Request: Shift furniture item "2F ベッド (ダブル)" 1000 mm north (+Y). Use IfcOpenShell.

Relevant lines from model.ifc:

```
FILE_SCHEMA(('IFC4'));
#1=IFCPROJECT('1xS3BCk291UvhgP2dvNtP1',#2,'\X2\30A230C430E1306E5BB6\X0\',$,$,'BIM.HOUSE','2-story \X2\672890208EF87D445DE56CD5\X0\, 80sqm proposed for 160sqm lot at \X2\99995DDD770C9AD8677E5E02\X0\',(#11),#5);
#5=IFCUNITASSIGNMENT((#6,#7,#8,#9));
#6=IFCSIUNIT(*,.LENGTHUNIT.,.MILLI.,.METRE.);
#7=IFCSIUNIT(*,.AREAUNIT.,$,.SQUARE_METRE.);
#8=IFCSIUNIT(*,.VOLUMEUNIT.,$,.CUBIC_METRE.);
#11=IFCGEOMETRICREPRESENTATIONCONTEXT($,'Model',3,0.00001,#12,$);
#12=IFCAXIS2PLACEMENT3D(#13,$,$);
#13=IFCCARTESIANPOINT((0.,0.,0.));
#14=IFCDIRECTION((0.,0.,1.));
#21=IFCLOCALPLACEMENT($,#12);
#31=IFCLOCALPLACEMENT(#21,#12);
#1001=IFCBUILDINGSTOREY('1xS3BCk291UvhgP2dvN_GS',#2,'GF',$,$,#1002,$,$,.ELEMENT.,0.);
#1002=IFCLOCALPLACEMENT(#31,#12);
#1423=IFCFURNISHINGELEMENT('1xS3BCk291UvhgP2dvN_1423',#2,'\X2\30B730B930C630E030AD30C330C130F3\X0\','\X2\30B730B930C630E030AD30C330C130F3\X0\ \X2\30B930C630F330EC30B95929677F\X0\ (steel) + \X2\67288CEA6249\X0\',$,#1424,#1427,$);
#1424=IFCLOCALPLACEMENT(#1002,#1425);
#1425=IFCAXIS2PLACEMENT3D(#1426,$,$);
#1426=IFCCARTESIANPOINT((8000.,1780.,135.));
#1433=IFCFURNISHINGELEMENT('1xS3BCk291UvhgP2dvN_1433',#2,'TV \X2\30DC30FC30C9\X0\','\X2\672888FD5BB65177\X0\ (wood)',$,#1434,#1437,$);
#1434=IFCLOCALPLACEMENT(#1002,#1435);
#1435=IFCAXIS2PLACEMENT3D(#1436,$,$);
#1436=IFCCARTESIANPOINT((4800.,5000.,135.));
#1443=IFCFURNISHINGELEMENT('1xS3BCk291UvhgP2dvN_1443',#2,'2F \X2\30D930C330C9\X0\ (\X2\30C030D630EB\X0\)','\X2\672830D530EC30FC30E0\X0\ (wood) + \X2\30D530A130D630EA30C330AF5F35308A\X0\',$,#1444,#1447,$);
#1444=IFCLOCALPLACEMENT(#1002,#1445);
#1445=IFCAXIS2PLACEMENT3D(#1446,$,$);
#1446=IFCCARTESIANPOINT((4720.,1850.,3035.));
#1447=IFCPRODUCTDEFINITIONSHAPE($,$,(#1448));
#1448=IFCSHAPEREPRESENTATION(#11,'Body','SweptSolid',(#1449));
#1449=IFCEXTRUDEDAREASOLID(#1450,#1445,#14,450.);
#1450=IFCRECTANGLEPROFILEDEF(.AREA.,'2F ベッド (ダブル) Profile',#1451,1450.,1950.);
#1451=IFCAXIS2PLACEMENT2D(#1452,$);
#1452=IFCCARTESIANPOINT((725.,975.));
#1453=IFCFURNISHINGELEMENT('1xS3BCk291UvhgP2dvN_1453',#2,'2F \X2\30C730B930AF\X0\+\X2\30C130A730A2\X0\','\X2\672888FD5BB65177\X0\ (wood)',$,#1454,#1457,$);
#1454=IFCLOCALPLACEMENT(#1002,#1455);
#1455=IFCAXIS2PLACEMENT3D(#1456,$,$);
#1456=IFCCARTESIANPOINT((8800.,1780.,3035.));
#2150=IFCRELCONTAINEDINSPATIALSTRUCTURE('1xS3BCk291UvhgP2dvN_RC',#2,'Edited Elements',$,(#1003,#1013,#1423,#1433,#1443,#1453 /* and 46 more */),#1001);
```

```python
import ifcopenshell
import ifcopenshell.api.geometry
import ifcopenshell.util.placement

model = ifcopenshell.open("model.ifc")

item = model.by_id(1443)
matrix = ifcopenshell.util.placement.get_local_placement(item.ObjectPlacement)
matrix[1, 3] += 1000.0
ifcopenshell.api.geometry.edit_object_placement(model, product=item, matrix=matrix, is_si=False)

print(ifcopenshell.util.placement.get_local_placement(item.ObjectPlacement).round(3) + 0.0)

model.write("model_updated.ifc")
```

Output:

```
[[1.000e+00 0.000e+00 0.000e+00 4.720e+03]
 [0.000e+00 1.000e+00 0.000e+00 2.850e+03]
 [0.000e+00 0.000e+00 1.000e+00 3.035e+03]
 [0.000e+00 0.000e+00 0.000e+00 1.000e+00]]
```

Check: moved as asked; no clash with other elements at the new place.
